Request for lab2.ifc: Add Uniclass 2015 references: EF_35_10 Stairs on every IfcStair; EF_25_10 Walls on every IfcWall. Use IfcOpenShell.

First a look at what the model holds.

```python
import ifcopenshell

model = ifcopenshell.open("lab2.ifc")
print(model.schema)
print("classifications:", [c.Name for c in model.by_type("IfcClassification")])
for ifc_class in ("IfcDoor", "IfcRoof", "IfcStair", "IfcWall", "IfcWindow"):
    print(ifc_class, len(model.by_type(ifc_class)))
```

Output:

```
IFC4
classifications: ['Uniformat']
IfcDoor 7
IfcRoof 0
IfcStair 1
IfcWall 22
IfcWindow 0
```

```python
import ifcopenshell
import ifcopenshell.api.classification

model = ifcopenshell.open("lab2.ifc")

system = ifcopenshell.api.classification.add_classification(model, classification="Uniclass 2015")

codes = {
    "IfcStair": ("EF_35_10", "Stairs"),
    "IfcWall": ("EF_25_10", "Walls"),
}
for ifc_class, (code, name) in codes.items():
    products = model.by_type(ifc_class)
    ifcopenshell.api.classification.add_reference(
        model, products=products, classification=system, identification=code, name=name
    )
    print(code, len(products))

model.write("lab2_rev.ifc")
```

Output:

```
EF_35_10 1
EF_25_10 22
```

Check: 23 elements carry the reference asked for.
